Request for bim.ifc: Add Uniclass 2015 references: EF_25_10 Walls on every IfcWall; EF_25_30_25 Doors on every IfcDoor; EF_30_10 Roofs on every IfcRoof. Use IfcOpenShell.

First a look at what the model holds.

```python
import ifcopenshell

model = ifcopenshell.open("bim.ifc")
print(model.schema)
print("classifications:", [c.Name for c in model.by_type("IfcClassification")])
for ifc_class in ("IfcDoor", "IfcRoof", "IfcStair", "IfcWall", "IfcWindow"):
    print(ifc_class, len(model.by_type(ifc_class)))
```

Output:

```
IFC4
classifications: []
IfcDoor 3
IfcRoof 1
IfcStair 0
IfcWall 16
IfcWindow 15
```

```python
import ifcopenshell
import ifcopenshell.api.classification

model = ifcopenshell.open("bim.ifc")

system = ifcopenshell.api.classification.add_classification(model, classification="Uniclass 2015")

codes = {
    "IfcWall": ("EF_25_10", "Walls"),
    "IfcDoor": ("EF_25_30_25", "Doors"),
    "IfcRoof": ("EF_30_10", "Roofs"),
}
for ifc_class, (code, name) in codes.items():
    products = model.by_type(ifc_class)
    ifcopenshell.api.classification.add_reference(
        model, products=products, classification=system, identification=code, name=name
    )
    print(code, len(products))

model.write("bim-out.ifc")
```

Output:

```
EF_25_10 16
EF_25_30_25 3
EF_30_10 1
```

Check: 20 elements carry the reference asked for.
